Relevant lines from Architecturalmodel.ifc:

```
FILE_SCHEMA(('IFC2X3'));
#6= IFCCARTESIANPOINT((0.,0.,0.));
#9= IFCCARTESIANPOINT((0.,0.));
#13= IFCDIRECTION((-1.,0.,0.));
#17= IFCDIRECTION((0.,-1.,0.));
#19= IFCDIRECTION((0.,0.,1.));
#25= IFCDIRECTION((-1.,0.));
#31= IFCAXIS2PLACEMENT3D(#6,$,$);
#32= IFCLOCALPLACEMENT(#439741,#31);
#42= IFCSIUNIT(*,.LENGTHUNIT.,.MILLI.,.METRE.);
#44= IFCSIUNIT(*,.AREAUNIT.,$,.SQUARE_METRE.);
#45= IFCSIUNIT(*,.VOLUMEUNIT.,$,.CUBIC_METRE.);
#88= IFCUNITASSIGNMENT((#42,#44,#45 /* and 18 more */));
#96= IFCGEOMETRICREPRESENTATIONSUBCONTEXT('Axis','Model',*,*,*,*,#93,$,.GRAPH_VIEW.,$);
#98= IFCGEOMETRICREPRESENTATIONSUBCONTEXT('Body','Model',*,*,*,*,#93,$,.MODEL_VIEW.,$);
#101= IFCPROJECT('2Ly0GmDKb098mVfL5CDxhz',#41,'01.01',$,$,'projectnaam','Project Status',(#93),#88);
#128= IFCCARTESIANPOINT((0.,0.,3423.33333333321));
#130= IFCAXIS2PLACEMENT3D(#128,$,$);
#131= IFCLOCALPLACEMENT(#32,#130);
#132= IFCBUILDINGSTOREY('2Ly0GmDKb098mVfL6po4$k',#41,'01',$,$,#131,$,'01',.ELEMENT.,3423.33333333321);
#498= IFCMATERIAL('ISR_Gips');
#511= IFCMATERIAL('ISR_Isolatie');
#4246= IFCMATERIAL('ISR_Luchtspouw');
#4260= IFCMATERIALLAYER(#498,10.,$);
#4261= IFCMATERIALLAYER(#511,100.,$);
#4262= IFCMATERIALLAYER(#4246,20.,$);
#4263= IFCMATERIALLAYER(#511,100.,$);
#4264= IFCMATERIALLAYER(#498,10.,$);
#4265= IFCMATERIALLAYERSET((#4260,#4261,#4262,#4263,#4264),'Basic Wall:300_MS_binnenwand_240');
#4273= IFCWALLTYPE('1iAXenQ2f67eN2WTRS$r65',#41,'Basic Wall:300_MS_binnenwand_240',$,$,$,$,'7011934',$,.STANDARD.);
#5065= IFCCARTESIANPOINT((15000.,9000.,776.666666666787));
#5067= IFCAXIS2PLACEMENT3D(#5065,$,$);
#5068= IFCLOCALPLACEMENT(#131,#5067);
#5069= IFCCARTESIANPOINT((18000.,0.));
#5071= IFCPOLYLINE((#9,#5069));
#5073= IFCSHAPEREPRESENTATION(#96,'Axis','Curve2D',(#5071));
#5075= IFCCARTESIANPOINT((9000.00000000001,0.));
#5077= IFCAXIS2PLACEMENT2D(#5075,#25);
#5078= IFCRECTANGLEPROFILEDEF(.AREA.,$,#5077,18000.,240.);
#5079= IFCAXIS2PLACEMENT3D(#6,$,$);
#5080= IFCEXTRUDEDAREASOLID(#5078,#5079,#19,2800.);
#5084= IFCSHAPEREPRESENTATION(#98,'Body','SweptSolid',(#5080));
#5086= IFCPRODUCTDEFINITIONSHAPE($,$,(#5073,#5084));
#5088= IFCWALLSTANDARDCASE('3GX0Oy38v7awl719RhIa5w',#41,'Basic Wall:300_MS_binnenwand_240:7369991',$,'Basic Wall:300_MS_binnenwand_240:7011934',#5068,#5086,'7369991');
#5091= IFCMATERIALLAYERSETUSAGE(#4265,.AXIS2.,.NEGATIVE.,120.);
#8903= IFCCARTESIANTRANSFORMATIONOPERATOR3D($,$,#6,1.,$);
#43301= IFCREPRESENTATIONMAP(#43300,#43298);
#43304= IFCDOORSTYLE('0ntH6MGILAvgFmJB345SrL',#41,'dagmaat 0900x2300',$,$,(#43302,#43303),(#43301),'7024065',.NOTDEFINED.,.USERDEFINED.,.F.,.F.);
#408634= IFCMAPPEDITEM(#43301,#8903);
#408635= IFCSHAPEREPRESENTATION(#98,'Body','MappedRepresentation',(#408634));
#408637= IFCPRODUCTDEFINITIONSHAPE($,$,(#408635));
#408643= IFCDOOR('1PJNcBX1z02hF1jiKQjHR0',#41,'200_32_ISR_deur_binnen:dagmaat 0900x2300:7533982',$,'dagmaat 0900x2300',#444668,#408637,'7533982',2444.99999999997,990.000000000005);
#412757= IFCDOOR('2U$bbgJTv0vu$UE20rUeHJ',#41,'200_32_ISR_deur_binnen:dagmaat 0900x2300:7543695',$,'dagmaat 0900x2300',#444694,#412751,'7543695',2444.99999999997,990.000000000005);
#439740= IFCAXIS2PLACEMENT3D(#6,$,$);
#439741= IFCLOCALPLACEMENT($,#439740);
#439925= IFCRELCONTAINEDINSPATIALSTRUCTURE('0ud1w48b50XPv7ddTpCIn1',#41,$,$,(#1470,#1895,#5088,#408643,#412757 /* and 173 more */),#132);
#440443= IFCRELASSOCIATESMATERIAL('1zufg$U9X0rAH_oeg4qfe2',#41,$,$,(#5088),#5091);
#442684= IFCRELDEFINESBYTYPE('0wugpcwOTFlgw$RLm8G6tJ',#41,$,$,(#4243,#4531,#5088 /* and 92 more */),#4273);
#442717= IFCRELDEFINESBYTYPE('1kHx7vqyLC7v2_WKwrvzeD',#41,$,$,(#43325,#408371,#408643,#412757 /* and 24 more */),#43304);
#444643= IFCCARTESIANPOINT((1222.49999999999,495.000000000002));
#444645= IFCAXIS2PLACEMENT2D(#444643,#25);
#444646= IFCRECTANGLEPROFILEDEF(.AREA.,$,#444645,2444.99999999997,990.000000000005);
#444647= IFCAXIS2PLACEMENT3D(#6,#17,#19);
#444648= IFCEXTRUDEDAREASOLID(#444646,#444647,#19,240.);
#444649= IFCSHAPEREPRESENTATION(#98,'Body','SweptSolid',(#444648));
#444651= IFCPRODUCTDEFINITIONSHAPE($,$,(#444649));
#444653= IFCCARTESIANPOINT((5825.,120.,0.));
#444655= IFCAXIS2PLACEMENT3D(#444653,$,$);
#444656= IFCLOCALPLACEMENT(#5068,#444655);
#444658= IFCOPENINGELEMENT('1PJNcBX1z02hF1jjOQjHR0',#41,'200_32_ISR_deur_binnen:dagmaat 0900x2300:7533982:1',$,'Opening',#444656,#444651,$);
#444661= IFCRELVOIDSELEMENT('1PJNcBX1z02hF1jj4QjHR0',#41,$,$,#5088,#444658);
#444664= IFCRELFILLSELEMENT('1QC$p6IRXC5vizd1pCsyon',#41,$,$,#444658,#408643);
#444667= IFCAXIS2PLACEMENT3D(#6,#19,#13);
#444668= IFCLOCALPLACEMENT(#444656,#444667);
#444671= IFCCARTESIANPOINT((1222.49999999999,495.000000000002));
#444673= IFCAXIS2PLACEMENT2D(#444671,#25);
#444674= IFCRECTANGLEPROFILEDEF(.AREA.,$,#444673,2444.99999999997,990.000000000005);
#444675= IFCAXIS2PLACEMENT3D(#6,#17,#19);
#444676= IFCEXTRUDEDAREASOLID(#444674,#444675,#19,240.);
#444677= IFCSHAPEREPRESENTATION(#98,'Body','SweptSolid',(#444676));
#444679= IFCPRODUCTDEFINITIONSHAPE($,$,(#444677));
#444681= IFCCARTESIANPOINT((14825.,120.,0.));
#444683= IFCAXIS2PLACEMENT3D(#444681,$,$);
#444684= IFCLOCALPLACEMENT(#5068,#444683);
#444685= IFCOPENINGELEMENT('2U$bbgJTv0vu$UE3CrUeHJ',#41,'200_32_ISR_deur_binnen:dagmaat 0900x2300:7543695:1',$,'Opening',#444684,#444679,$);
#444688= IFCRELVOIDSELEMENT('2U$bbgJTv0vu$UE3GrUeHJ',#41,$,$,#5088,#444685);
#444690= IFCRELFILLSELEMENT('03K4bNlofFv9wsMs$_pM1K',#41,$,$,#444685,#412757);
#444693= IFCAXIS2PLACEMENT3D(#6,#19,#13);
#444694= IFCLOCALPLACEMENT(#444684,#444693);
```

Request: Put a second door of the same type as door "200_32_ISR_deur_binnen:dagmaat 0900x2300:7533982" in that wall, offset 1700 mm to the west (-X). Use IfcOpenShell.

```python
import ifcopenshell
import ifcopenshell.api.feature
import ifcopenshell.api.geometry
import ifcopenshell.api.root
import ifcopenshell.geom
import ifcopenshell.util.element
import ifcopenshell.util.placement
import ifcopenshell.util.shape

model = ifcopenshell.open("Architecturalmodel.ifc")
settings = ifcopenshell.geom.settings()


def volume(element):
    """Net volume in cubic metres, openings subtracted."""
    shape = ifcopenshell.geom.create_shape(settings, element)
    return ifcopenshell.util.shape.get_volume(shape.geometry)


def reuse_history(source, copy):
    """copy_class also copies each property set's owner history, people and application; keep the originals."""
    for rel in copy.IsDefinedBy:
        if rel.is_a("IfcRelDefinesByProperties") and (history := rel.RelatingPropertyDefinition.OwnerHistory):
            rel.RelatingPropertyDefinition.OwnerHistory = source.OwnerHistory
            ifcopenshell.util.element.remove_deep2(model, history)


door = model.by_id(408643)
opening = door.FillsVoids[0].RelatingOpeningElement
wall = opening.VoidsElements[0].RelatingBuildingElement
before = volume(wall)
shift = ifcopenshell.util.placement.get_local_placement(wall.ObjectPlacement)[:3, 0] * -1700.0

# copy_class copies the void relationship, type, container and properties, but no geometry.
new_opening = ifcopenshell.api.root.copy_class(model, product=opening)
new_opening.Representation = ifcopenshell.util.element.copy_deep(
    model, opening.Representation, exclude=["IfcGeometricRepresentationContext", "IfcRepresentationMap"]
)
new_opening.Name = "200_32_ISR_deur_binnen:dagmaat 0900x2300"
new_door = ifcopenshell.api.root.copy_class(model, product=door)
new_door.Representation = ifcopenshell.util.element.copy_deep(
    model, door.Representation, exclude=["IfcGeometricRepresentationContext", "IfcRepresentationMap"]
)
new_door.Name = "200_32_ISR_deur_binnen:dagmaat 0900x2300"
new_door.Tag = None
reuse_history(door, new_door)
fills = ifcopenshell.api.feature.add_filling(model, opening=new_opening, element=new_door)
fills.OwnerHistory = new_door.OwnerHistory  # required in IFC2X3

for old, new in ((opening, new_opening), (door, new_door)):
    matrix = ifcopenshell.util.placement.get_local_placement(old.ObjectPlacement)
    matrix[:3, 3] += shift
    ifcopenshell.api.geometry.edit_object_placement(model, product=new, matrix=matrix, is_si=False)

after = volume(wall)

print(f"wall volume {before:.3f} -> {after:.3f} m3")

model.write("Architecturalmodel-out.ifc")
```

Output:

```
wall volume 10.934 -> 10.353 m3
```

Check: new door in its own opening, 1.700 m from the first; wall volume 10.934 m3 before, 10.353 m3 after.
